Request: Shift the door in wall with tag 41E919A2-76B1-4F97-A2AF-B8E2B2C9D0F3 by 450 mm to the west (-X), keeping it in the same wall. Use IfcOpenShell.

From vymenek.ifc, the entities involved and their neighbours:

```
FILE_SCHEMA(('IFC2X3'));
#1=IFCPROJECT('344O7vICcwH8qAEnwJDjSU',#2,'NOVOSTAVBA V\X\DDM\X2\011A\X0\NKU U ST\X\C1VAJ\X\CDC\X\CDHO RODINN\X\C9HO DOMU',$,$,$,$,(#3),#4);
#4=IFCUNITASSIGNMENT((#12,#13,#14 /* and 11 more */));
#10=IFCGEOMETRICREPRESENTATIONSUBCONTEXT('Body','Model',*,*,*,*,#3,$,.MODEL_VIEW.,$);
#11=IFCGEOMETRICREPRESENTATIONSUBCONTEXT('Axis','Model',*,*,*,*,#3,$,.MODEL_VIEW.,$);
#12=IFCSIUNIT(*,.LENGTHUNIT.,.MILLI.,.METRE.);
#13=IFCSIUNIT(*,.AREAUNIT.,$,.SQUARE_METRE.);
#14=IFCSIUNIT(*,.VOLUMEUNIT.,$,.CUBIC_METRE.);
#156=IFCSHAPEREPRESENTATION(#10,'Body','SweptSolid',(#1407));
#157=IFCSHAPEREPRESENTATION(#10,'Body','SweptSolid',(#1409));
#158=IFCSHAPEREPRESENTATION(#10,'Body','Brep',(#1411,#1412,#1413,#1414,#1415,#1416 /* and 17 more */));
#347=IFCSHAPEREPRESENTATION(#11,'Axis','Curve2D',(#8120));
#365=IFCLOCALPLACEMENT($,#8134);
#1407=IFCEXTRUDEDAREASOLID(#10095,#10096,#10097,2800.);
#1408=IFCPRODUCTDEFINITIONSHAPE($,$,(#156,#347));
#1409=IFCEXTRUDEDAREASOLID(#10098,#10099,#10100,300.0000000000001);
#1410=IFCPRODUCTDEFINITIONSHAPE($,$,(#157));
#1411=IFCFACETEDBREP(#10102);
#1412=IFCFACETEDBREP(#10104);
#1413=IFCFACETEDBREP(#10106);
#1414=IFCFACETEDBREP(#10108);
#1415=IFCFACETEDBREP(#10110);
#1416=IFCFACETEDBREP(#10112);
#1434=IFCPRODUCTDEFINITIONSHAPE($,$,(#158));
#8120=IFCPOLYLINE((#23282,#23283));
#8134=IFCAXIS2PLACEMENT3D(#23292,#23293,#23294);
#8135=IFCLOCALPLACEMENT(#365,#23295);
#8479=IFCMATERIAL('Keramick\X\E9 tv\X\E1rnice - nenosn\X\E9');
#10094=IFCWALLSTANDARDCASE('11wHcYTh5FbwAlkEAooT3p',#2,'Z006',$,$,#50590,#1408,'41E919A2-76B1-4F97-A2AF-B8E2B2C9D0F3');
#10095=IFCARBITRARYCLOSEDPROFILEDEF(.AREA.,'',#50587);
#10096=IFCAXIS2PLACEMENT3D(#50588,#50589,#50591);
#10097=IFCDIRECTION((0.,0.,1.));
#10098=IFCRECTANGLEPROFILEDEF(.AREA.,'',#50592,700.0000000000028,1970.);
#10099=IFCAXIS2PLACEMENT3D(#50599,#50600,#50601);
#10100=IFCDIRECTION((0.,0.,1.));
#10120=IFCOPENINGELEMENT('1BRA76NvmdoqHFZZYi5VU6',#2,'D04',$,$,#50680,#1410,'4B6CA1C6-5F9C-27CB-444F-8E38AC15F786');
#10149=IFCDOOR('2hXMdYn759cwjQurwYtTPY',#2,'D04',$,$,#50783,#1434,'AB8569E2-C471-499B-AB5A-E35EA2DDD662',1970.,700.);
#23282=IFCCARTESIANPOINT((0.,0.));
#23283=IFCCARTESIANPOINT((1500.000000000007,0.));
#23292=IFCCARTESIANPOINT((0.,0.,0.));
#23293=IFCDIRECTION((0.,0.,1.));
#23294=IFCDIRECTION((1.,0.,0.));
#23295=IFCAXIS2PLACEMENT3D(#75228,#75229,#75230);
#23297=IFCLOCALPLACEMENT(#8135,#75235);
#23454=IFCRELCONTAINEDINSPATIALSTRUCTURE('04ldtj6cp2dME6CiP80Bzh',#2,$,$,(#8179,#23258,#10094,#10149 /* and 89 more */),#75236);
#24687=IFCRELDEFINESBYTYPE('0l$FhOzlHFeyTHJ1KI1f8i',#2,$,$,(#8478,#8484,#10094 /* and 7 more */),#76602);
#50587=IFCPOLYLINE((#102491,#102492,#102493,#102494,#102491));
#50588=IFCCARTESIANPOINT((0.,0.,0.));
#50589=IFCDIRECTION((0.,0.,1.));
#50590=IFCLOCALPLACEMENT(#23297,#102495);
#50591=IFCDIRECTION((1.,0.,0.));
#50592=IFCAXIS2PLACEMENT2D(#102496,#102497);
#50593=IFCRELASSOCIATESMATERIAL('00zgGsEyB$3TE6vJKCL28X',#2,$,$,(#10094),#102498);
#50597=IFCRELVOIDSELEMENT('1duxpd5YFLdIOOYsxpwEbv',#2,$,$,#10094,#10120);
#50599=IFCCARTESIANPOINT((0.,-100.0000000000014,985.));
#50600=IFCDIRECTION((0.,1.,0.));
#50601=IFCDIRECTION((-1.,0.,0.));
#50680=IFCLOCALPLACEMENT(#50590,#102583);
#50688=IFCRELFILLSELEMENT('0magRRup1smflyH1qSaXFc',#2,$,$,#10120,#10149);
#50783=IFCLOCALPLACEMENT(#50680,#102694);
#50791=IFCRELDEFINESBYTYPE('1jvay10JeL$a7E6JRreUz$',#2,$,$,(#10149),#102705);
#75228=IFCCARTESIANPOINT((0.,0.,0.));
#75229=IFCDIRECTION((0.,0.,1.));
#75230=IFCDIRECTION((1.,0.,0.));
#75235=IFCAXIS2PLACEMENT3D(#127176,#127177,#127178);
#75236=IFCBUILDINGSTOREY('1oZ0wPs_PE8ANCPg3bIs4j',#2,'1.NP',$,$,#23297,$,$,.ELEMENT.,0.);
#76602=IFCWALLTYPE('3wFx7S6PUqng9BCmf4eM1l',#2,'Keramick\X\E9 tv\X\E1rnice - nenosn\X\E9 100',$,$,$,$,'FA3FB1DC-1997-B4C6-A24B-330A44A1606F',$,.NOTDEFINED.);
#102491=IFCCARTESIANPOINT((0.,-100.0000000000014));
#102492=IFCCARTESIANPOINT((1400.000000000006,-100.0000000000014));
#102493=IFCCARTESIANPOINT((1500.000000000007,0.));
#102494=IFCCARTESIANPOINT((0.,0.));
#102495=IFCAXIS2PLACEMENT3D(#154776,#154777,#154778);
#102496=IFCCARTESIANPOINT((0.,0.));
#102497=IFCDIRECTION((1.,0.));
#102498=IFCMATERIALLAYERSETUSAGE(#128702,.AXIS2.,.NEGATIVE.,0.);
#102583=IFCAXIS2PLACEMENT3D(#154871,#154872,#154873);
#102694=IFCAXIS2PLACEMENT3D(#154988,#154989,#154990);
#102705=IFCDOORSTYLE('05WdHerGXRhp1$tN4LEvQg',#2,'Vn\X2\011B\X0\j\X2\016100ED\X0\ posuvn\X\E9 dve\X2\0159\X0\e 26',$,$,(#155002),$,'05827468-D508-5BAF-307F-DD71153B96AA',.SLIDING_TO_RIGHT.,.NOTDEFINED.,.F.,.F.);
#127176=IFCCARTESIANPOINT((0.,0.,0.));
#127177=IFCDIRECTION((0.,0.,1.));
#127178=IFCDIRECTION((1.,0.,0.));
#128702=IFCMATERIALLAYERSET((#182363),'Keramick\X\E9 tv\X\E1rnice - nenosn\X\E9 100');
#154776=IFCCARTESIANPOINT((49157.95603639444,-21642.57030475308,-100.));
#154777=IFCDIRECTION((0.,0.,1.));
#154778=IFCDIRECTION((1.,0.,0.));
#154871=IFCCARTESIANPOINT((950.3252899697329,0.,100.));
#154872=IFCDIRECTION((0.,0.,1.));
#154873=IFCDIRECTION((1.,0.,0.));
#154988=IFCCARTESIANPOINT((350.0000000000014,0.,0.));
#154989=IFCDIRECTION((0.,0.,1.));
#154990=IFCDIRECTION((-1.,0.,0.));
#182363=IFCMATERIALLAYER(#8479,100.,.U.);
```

```python
import ifcopenshell
import ifcopenshell.api.geometry
import ifcopenshell.util.placement
import ifcopenshell.util.unit

model = ifcopenshell.open("vymenek.ifc")
unit_scale = ifcopenshell.util.unit.calculate_unit_scale(model)

door = model.by_guid("2hXMdYn759cwjQurwYtTPY")
opening = door.FillsVoids[0].RelatingOpeningElement
wall = opening.VoidsElements[0].RelatingBuildingElement

wall_matrix = ifcopenshell.util.placement.get_local_placement(wall.ObjectPlacement)
shift = wall_matrix[:3, 0] * -0.45 / unit_scale
before = ifcopenshell.util.placement.get_local_placement(door.ObjectPlacement)[:3, 3].copy()

# The door is placed relative to its opening, so it follows when the opening moves.
matrix = ifcopenshell.util.placement.get_local_placement(opening.ObjectPlacement)
matrix[:3, 3] += shift
ifcopenshell.api.geometry.edit_object_placement(
    model, product=opening, matrix=matrix, is_si=False, should_transform_children=True
)

after = ifcopenshell.util.placement.get_local_placement(door.ObjectPlacement)[:3, 3]
print("door moved by", (after - before).round(3) + 0.0)

model.write("vymenek_rev.ifc")
```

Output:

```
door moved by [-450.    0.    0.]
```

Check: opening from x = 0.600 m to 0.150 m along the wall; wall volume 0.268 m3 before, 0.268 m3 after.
